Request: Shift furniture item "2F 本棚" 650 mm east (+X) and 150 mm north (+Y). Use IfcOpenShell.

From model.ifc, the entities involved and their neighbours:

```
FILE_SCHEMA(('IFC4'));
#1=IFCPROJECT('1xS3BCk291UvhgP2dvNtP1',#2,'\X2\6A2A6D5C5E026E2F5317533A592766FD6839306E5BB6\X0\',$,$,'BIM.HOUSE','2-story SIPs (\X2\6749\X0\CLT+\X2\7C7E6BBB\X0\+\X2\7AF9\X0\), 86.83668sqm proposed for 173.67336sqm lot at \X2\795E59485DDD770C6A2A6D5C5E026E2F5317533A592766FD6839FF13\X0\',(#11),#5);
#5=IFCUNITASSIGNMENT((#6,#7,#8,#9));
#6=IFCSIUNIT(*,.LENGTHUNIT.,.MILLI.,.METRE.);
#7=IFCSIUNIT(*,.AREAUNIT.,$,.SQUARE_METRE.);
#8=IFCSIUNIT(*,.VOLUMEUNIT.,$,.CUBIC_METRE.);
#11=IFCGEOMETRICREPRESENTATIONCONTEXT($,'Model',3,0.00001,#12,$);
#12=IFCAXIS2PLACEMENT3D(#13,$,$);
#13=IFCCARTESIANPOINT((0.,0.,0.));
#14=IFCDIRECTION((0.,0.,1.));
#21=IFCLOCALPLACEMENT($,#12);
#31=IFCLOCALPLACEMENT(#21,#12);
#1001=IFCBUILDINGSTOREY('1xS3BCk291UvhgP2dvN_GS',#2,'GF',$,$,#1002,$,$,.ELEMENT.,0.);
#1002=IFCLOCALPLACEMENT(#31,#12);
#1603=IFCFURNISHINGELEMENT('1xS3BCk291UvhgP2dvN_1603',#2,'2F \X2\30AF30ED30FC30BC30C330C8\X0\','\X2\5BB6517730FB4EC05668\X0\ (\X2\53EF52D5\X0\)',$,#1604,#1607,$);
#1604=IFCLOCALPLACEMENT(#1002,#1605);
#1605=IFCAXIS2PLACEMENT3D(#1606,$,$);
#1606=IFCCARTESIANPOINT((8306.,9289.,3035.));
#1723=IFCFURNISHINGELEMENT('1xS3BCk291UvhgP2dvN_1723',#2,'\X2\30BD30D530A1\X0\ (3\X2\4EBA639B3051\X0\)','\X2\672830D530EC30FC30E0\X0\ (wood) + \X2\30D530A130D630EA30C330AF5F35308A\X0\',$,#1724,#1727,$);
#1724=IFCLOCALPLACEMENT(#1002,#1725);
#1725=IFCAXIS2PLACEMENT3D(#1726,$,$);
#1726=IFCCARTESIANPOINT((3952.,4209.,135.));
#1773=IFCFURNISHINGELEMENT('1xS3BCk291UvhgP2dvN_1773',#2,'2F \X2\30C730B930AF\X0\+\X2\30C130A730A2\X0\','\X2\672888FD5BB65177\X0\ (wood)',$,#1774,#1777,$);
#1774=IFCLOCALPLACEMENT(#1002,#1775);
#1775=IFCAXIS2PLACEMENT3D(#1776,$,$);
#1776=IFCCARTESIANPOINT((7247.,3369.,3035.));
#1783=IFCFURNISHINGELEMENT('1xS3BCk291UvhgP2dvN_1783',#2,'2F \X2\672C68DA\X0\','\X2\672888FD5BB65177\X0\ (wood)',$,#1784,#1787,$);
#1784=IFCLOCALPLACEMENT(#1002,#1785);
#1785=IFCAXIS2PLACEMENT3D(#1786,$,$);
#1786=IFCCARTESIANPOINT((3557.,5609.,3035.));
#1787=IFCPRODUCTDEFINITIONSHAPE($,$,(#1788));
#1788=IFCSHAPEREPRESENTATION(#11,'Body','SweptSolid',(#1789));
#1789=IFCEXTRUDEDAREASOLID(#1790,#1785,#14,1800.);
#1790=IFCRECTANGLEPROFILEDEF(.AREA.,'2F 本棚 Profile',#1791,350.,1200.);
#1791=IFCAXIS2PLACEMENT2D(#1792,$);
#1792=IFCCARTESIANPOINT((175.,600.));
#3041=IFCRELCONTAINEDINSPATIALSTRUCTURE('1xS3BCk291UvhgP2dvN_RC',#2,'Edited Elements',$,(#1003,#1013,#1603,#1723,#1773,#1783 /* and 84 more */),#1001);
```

```python
import ifcopenshell
import ifcopenshell.api.geometry
import ifcopenshell.util.placement
import ifcopenshell.util.unit

model = ifcopenshell.open("model.ifc")
unit_scale = ifcopenshell.util.unit.calculate_unit_scale(model)

item = model.by_guid("1xS3BCk291UvhgP2dvN_1783")
matrix = ifcopenshell.util.placement.get_local_placement(item.ObjectPlacement)
matrix[0, 3] += 0.65 / unit_scale
matrix[1, 3] += 0.15 / unit_scale
ifcopenshell.api.geometry.edit_object_placement(model, product=item, matrix=matrix, is_si=False)

print(ifcopenshell.util.placement.get_local_placement(item.ObjectPlacement).round(3) + 0.0)

model.write("model_v2.ifc")
```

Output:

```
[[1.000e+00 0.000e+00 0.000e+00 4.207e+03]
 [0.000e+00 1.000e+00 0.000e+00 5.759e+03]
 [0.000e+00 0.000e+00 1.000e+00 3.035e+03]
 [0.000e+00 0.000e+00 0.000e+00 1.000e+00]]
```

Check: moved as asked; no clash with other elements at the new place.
